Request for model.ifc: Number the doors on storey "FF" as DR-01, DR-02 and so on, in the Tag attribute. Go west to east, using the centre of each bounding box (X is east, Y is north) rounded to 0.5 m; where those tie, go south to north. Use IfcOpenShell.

First a look at what the model holds.

```python
import ifcopenshell
import ifcopenshell.util.element
import ifcopenshell.util.placement

model = ifcopenshell.open("model.ifc")
print(model.schema)
storey = next(s for s in model.by_type("IfcBuildingStorey") if s.Name == "FF")
doors = [e for e in ifcopenshell.util.element.get_decomposition(storey) if e.is_a("IfcDoor")]
for e in sorted(doors, key=lambda e: e.id()):
    origin = ifcopenshell.util.placement.get_local_placement(e.ObjectPlacement)[:3, 3]
    print(e.id(), e.Tag, e.Name, origin.round(2) + 0.0, sep=" | ")
```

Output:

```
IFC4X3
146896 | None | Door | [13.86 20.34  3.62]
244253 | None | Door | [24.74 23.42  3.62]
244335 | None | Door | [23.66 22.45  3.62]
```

```python
import ifcopenshell
import ifcopenshell.geom
import ifcopenshell.util.element
import ifcopenshell.util.shape

model = ifcopenshell.open("model.ifc")
settings = ifcopenshell.geom.settings()
settings.set("use-world-coords", True)


def centre(element):
    shape = ifcopenshell.geom.create_shape(settings, element)
    return ifcopenshell.util.shape.get_bbox_centroid(shape.geometry)


storey = next(s for s in model.by_type("IfcBuildingStorey") if s.Name == "FF")
doors = [e for e in ifcopenshell.util.element.get_decomposition(storey) if e.is_a("IfcDoor")]

# Insertion points can sit at a corner or the storey origin, so sort by the geometry (in metres).
centres = {e: centre(e) for e in doors}
doors.sort(key=lambda e: (round(centres[e][0] / 0.5), centres[e][1]))

for i, e in enumerate(doors, start=1):
    number = f"DR-{i:02d}"
    e.Tag = number
    print(e.id(), number)

model.write("model_rev.ifc")
```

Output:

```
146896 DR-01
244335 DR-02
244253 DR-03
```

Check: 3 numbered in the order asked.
